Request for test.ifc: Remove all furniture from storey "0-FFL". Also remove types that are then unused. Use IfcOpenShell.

First a look at what the model holds.

```python
import ifcopenshell
import ifcopenshell.util.element

model = ifcopenshell.open("test.ifc")
print(model.schema)
storey = next(s for s in model.by_type("IfcBuildingStorey") if s.Name == "0-FFL")
furniture = [e for e in ifcopenshell.util.element.get_decomposition(storey) if e.is_a("IfcFurnishingElement")]
seen = {}
for e in furniture:
    element_type = ifcopenshell.util.element.get_type(e)
    name = element_type.Name if element_type not in (None, e) else None
    seen[name] = seen.get(name, 0) + 1
for name, count in sorted(seen.items(), key=str):
    print(count, "x", name)
```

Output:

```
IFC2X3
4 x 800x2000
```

```python
import ifcopenshell
import ifcopenshell.api.root
import ifcopenshell.util.element

model = ifcopenshell.open("test.ifc")

storey = next(s for s in model.by_type("IfcBuildingStorey") if s.Name == "0-FFL")
furniture = [e for e in ifcopenshell.util.element.get_decomposition(storey) if e.is_a("IfcFurnishingElement")]
types = {ifcopenshell.util.element.get_type(e) for e in furniture} - {None, *furniture}

for e in furniture:
    ifcopenshell.api.root.remove_product(model, product=e)
print(len(furniture), "removed")

unused = [t for t in types if not ifcopenshell.util.element.get_types(t)]
for t in unused:
    ifcopenshell.api.root.remove_product(model, product=t)
print(len(unused), "unused types removed")

model.write("test-out.ifc")
```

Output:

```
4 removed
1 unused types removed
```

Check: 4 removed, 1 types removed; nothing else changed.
